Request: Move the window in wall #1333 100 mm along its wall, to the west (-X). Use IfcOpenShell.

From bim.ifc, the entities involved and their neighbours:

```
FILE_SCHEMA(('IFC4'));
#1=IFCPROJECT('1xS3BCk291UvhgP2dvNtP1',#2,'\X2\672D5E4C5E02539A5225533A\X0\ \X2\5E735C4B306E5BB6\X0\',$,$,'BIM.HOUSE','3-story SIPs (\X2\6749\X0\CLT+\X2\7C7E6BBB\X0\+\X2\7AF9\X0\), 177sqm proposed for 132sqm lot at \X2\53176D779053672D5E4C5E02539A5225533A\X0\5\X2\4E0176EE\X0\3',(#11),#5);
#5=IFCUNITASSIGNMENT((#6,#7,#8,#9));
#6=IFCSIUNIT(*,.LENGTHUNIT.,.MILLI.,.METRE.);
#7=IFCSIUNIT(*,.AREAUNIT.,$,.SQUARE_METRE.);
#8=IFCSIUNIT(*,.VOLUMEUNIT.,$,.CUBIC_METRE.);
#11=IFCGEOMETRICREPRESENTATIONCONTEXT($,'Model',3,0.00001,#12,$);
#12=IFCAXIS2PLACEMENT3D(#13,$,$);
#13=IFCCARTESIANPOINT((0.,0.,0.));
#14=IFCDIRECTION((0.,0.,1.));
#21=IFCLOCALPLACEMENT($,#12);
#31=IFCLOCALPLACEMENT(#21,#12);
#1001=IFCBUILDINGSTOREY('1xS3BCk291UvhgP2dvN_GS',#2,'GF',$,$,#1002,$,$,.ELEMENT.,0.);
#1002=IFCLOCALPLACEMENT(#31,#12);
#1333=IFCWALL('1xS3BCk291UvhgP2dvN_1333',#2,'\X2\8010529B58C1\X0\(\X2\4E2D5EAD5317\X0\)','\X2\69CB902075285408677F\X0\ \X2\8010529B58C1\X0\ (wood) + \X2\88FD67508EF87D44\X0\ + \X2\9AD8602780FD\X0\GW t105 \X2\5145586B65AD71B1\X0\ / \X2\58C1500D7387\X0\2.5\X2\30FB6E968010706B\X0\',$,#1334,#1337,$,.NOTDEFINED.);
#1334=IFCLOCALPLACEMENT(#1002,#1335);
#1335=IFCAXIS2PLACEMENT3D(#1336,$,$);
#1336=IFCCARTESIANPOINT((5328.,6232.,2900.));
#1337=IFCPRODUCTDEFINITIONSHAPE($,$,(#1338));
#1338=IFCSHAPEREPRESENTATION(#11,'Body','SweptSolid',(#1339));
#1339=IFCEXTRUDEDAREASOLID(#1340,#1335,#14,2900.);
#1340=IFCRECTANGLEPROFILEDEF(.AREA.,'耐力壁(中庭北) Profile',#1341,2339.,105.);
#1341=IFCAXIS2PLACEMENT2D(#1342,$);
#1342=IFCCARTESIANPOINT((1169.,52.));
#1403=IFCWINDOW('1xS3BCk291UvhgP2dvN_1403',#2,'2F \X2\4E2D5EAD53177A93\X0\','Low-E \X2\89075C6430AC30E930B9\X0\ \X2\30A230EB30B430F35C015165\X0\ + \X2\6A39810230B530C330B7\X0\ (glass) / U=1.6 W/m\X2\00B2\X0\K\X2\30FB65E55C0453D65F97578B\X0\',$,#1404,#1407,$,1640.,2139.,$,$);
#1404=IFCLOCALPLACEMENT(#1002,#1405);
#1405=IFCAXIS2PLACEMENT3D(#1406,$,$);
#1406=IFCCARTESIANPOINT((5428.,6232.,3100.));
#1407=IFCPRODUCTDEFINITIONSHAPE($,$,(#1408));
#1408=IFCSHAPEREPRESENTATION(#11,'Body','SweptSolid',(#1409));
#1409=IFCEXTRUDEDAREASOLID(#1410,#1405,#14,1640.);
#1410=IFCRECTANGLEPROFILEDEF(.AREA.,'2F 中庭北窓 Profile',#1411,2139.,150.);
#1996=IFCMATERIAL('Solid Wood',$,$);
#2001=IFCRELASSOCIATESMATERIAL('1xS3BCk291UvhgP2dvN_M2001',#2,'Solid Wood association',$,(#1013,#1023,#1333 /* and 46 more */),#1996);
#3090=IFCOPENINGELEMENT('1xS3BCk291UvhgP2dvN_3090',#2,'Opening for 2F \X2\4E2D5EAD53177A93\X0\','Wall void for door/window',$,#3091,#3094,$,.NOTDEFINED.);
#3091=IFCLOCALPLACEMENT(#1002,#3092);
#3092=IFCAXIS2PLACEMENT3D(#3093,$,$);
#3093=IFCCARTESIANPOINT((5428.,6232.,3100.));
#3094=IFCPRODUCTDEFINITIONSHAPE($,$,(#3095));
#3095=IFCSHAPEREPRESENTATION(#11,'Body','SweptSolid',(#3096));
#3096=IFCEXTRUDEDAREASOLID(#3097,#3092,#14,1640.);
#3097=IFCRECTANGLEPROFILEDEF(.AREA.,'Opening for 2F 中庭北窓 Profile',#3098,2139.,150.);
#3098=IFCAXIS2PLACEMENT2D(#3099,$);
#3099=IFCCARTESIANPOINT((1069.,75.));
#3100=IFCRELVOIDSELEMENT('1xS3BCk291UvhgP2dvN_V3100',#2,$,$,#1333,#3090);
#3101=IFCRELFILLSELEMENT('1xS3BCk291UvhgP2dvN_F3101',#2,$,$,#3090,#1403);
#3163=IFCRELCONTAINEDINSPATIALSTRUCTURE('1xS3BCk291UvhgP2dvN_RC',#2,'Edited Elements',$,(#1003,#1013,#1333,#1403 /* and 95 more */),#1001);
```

```python
import ifcopenshell
import ifcopenshell.api.geometry
import ifcopenshell.util.placement
import ifcopenshell.util.unit

model = ifcopenshell.open("bim.ifc")
unit_scale = ifcopenshell.util.unit.calculate_unit_scale(model)

window = model.by_guid("1xS3BCk291UvhgP2dvN_1403")
opening = window.FillsVoids[0].RelatingOpeningElement
wall = opening.VoidsElements[0].RelatingBuildingElement

wall_matrix = ifcopenshell.util.placement.get_local_placement(wall.ObjectPlacement)
shift = wall_matrix[:3, 0] * -0.1 / unit_scale
before = ifcopenshell.util.placement.get_local_placement(window.ObjectPlacement)[:3, 3].copy()

# The window is not placed relative to its opening, so move both.
for product in (opening, window):
    matrix = ifcopenshell.util.placement.get_local_placement(product.ObjectPlacement)
    matrix[:3, 3] += shift
    ifcopenshell.api.geometry.edit_object_placement(model, product=product, matrix=matrix, is_si=False)

after = ifcopenshell.util.placement.get_local_placement(window.ObjectPlacement)[:3, 3]
print("window moved by", (after - before).round(3) + 0.0)

model.write("bim_edited.ifc")
```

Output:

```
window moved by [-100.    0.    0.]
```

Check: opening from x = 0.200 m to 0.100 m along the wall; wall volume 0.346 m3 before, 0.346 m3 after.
